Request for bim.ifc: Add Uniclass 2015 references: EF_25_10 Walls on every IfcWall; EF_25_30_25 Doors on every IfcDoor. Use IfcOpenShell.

First a look at what the model holds.

```python
import ifcopenshell

model = ifcopenshell.open("bim.ifc")
print(model.schema)
print("classifications:", [c.Name for c in model.by_type("IfcClassification")])
for ifc_class in ("IfcDoor", "IfcRoof", "IfcStair", "IfcWall", "IfcWindow"):
    print(ifc_class, len(model.by_type(ifc_class)))
```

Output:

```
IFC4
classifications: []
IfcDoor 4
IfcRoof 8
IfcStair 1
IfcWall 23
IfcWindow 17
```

```python
import ifcopenshell
import ifcopenshell.api.classification

model = ifcopenshell.open("bim.ifc")

system = ifcopenshell.api.classification.add_classification(model, classification="Uniclass 2015")

codes = {
    "IfcWall": ("EF_25_10", "Walls"),
    "IfcDoor": ("EF_25_30_25", "Doors"),
}
for ifc_class, (code, name) in codes.items():
    products = model.by_type(ifc_class)
    ifcopenshell.api.classification.add_reference(
        model, products=products, classification=system, identification=code, name=name
    )
    print(code, len(products))

model.write("bim-out.ifc")
```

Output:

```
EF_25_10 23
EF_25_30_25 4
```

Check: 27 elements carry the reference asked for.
